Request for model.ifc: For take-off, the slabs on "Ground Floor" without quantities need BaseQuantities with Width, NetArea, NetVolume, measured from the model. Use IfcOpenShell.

First a look at what the model holds.

```python
import ifcopenshell
import ifcopenshell.util.element
import ifcopenshell.util.unit

model = ifcopenshell.open("model.ifc")
print(model.schema)
for unit_type in ("LENGTHUNIT", "AREAUNIT", "VOLUMEUNIT"):
    print(unit_type, ifcopenshell.util.unit.calculate_unit_scale(model, unit_type))
storey = next(s for s in model.by_type("IfcBuildingStorey") if s.Name == "Ground Floor")
slabs = [e for e in ifcopenshell.util.element.get_decomposition(storey) if e.is_a("IfcSlab")]
for e in sorted(slabs, key=lambda e: e.id()):
    print(e.id(), e.is_a(), e.Name, list(ifcopenshell.util.element.get_psets(e, qtos_only=True)), sep=" | ")
```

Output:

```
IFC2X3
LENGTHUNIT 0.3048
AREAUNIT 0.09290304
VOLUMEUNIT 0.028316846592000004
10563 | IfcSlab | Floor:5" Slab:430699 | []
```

```python
import ifcopenshell
import ifcopenshell.api.pset
import ifcopenshell.geom
import ifcopenshell.util.element
import ifcopenshell.util.shape
import ifcopenshell.util.unit

model = ifcopenshell.open("model.ifc")
unit_scale = ifcopenshell.util.unit.calculate_unit_scale(model)
area_scale = ifcopenshell.util.unit.calculate_unit_scale(model, "AREAUNIT")
volume_scale = ifcopenshell.util.unit.calculate_unit_scale(model, "VOLUMEUNIT")
settings = ifcopenshell.geom.settings()

storey = next(s for s in model.by_type("IfcBuildingStorey") if s.Name == "Ground Floor")
slabs = [e for e in ifcopenshell.util.element.get_decomposition(storey) if e.is_a("IfcSlab")]

for e in sorted(slabs, key=lambda e: e.id()):
    if ifcopenshell.util.element.get_psets(e, qtos_only=True, should_inherit=False):
        continue
    # Geometry comes back in metres, in the element's own axes.
    shape = ifcopenshell.geom.create_shape(settings, e)
    values = {
        "Width": ifcopenshell.util.shape.get_z(shape.geometry) / unit_scale,
        "NetArea": ifcopenshell.util.shape.get_footprint_area(shape.geometry) / area_scale,
        "NetVolume": ifcopenshell.util.shape.get_volume(shape.geometry) / volume_scale,
    }
    qto = ifcopenshell.api.pset.add_qto(model, product=e, name="BaseQuantities")
    ifcopenshell.api.pset.edit_qto(model, qto=qto, properties=values)
    print(e.id(), {k: round(v, 3) for k, v in values.items()})

model.write("model-out.ifc")
```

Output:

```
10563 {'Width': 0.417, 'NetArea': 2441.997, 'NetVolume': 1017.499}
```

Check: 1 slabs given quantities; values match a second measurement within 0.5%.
